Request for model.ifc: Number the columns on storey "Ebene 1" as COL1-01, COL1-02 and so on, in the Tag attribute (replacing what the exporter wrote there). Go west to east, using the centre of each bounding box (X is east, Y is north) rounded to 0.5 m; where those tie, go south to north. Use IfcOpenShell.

First a look at what the model holds.

```python
import ifcopenshell
import ifcopenshell.util.element
import ifcopenshell.util.placement

model = ifcopenshell.open("model.ifc")
print(model.schema)
storey = next(s for s in model.by_type("IfcBuildingStorey") if s.Name == "Ebene 1")
columns = [e for e in ifcopenshell.util.element.get_decomposition(storey) if e.is_a("IfcColumn")]
for e in sorted(columns, key=lambda e: e.id()):
    origin = ifcopenshell.util.placement.get_local_placement(e.ObjectPlacement)[:3, 3]
    print(e.id(), e.Tag, e.Name, origin.round(2) + 0.0, sep=" | ")
```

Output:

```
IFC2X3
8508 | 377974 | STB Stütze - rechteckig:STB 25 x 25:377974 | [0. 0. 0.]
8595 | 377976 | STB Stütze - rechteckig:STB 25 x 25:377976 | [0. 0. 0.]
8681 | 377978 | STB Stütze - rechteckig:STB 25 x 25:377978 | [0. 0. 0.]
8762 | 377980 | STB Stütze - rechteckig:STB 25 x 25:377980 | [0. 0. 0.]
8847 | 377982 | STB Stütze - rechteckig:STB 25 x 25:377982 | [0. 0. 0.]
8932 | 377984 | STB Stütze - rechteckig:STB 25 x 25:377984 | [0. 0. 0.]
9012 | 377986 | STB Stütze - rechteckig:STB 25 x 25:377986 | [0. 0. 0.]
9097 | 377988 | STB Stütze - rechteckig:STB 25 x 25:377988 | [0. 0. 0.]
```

```python
import ifcopenshell
import ifcopenshell.geom
import ifcopenshell.util.element
import ifcopenshell.util.shape

model = ifcopenshell.open("model.ifc")
settings = ifcopenshell.geom.settings()
settings.set("use-world-coords", True)


def centre(element):
    shape = ifcopenshell.geom.create_shape(settings, element)
    return ifcopenshell.util.shape.get_bbox_centroid(shape.geometry)


storey = next(s for s in model.by_type("IfcBuildingStorey") if s.Name == "Ebene 1")
columns = [e for e in ifcopenshell.util.element.get_decomposition(storey) if e.is_a("IfcColumn")]

# Insertion points can sit at a corner or the storey origin, so sort by the geometry (in metres).
centres = {e: centre(e) for e in columns}
columns.sort(key=lambda e: (round(centres[e][0] / 0.5), centres[e][1]))

for i, e in enumerate(columns, start=1):
    number = f"COL1-{i:02d}"
    e.Tag = number
    print(e.id(), number)

model.write("model_updated.ifc")
```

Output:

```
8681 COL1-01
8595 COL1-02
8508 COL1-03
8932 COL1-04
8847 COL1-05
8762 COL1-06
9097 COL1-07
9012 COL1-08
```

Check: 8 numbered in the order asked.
